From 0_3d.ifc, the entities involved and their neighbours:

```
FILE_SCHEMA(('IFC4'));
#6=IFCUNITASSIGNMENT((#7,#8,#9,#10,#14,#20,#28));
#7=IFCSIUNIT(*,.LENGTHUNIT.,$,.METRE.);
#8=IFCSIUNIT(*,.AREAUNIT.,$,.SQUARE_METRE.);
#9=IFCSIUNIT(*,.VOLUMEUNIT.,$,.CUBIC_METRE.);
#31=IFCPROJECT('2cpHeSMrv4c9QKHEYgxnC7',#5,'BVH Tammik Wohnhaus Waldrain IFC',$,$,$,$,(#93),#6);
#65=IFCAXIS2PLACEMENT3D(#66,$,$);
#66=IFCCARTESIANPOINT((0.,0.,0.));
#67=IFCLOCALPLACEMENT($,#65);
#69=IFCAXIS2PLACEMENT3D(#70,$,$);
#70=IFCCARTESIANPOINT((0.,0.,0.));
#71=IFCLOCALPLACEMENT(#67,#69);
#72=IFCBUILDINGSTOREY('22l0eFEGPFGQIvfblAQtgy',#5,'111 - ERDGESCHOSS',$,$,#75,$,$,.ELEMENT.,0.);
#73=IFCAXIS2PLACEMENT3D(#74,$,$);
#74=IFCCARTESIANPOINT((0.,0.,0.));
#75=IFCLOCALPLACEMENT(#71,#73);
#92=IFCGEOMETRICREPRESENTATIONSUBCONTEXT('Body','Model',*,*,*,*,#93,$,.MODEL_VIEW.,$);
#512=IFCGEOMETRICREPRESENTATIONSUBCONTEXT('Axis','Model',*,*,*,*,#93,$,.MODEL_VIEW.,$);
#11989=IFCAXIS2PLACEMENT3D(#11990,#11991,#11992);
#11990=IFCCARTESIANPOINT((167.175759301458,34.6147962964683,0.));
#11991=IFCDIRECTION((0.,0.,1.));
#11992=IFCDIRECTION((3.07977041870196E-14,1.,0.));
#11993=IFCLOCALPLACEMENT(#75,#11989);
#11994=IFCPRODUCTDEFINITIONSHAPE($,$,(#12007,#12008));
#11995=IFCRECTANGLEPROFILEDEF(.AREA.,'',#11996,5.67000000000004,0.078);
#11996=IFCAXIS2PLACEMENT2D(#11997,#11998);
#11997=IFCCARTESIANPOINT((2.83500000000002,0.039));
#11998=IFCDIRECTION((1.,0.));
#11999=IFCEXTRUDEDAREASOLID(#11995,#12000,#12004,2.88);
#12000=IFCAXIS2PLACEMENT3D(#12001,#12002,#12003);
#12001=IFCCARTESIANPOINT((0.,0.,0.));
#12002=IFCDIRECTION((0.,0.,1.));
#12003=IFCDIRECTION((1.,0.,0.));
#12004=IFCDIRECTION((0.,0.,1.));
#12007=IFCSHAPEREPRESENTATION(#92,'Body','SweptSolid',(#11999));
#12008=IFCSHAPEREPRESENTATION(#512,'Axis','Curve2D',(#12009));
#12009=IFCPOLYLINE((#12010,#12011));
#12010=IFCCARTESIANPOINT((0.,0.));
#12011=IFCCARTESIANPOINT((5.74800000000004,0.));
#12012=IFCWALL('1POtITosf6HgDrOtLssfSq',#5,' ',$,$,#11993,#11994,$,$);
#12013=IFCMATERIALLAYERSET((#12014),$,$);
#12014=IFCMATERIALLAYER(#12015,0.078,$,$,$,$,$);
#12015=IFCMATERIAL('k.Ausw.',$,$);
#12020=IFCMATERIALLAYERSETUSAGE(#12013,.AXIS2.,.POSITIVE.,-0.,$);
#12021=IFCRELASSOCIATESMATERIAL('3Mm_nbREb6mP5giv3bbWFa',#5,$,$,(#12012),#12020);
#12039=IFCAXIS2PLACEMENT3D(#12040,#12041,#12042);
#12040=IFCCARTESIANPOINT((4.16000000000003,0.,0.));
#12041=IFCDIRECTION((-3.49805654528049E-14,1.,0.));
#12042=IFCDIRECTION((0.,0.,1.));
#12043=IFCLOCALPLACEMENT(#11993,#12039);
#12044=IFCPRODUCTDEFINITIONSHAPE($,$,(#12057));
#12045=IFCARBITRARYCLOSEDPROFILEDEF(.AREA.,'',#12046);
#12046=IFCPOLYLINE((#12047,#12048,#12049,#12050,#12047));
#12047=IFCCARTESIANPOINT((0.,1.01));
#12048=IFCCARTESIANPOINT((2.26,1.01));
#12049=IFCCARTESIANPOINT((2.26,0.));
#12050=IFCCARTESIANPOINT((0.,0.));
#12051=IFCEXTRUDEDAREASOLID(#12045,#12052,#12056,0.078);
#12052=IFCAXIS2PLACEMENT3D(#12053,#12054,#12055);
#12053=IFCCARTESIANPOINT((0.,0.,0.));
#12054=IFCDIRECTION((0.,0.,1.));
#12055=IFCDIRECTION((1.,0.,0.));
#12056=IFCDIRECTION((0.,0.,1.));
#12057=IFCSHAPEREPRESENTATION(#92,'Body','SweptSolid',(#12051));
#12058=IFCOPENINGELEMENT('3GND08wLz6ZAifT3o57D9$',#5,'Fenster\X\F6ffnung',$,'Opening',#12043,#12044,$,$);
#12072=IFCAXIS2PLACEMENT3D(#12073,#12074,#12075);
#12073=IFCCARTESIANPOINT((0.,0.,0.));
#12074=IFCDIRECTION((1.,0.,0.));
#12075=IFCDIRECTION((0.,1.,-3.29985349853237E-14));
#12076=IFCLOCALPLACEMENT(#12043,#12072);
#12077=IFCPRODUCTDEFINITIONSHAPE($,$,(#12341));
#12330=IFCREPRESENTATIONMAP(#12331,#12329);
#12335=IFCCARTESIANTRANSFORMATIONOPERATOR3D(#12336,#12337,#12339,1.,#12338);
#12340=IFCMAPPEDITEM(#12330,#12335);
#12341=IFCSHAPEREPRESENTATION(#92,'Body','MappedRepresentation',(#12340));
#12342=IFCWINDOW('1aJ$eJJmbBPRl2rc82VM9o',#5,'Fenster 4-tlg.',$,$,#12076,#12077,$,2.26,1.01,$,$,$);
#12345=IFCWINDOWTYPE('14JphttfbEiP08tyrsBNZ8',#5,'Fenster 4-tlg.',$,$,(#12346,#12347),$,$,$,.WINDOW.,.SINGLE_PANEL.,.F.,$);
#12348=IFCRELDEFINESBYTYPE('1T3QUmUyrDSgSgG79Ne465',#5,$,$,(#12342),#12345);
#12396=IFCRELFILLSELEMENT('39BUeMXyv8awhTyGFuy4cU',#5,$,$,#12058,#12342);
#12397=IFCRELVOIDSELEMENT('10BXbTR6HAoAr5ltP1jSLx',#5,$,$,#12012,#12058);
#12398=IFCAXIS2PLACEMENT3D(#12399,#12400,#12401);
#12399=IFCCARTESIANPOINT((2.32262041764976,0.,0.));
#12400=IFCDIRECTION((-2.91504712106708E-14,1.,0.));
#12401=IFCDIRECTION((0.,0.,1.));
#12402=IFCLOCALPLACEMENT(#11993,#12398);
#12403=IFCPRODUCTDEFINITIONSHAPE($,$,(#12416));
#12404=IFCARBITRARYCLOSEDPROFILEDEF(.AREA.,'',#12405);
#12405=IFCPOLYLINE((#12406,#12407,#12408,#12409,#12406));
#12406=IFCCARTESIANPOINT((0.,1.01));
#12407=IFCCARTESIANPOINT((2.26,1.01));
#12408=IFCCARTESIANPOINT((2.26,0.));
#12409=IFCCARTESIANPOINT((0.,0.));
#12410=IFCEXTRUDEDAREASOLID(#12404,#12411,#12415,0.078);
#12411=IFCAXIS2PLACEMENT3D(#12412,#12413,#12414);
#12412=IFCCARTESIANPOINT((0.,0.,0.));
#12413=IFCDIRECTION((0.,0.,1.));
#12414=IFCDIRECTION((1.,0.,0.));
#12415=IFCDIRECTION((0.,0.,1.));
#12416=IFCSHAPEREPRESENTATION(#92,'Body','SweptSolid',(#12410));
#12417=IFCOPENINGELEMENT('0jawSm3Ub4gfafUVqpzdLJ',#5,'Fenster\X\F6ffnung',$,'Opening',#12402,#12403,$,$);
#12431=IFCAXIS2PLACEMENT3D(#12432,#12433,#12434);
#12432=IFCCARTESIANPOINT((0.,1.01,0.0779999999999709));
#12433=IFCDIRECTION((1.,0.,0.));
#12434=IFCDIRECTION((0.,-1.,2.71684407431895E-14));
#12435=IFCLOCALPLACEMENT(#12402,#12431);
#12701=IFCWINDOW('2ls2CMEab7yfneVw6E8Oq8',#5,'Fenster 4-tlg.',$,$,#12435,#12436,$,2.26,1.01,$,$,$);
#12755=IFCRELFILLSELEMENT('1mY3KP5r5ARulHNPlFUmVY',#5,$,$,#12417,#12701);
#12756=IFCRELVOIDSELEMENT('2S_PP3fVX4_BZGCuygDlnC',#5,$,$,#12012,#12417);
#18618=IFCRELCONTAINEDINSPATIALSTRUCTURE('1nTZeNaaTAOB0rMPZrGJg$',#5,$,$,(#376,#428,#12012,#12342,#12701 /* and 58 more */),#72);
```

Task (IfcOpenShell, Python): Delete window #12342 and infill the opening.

```python
import ifcopenshell
import ifcopenshell.api.feature
import ifcopenshell.api.root
import ifcopenshell.geom
import ifcopenshell.util.shape

model = ifcopenshell.open("0_3d.ifc")
settings = ifcopenshell.geom.settings()


def volume(element):
    """Net volume in cubic metres, openings subtracted."""
    shape = ifcopenshell.geom.create_shape(settings, element)
    return ifcopenshell.util.shape.get_volume(shape.geometry)


window = model.by_guid("1aJ$eJJmbBPRl2rc82VM9o")
opening = window.FillsVoids[0].RelatingOpeningElement
wall = opening.VoidsElements[0].RelatingBuildingElement
before = volume(wall)

ifcopenshell.api.root.remove_product(model, product=window)
ifcopenshell.api.feature.remove_feature(model, feature=opening)

after = volume(wall)

print(f"wall volume {before:.3f} -> {after:.3f} m3")

model.write("0_3d_updated.ifc")
```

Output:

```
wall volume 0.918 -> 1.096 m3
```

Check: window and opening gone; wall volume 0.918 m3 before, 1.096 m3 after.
